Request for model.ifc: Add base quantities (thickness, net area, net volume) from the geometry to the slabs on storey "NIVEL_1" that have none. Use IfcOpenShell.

First a look at what the model holds.

```python
import ifcopenshell
import ifcopenshell.util.element
import ifcopenshell.util.unit

model = ifcopenshell.open("model.ifc")
print(model.schema)
for unit_type in ("LENGTHUNIT", "AREAUNIT", "VOLUMEUNIT"):
    print(unit_type, ifcopenshell.util.unit.calculate_unit_scale(model, unit_type))
storey = next(s for s in model.by_type("IfcBuildingStorey") if s.Name == "NIVEL_1")
slabs = [e for e in ifcopenshell.util.element.get_decomposition(storey) if e.is_a("IfcSlab")]
for e in sorted(slabs, key=lambda e: e.id()):
    print(e.id(), e.is_a(), e.Name, list(ifcopenshell.util.element.get_psets(e, qtos_only=True)), sep=" | ")
```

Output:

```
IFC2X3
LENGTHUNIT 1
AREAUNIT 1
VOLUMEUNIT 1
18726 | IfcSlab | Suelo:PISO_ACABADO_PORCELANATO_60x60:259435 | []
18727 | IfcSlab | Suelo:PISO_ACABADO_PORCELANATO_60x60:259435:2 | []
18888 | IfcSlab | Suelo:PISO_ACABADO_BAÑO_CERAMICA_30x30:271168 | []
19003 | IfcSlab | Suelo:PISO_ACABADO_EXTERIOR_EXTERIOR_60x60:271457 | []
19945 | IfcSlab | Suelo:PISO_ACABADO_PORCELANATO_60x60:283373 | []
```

```python
import ifcopenshell
import ifcopenshell.api.pset
import ifcopenshell.geom
import ifcopenshell.util.element
import ifcopenshell.util.shape
import ifcopenshell.util.unit

model = ifcopenshell.open("model.ifc")
unit_scale = ifcopenshell.util.unit.calculate_unit_scale(model)
area_scale = ifcopenshell.util.unit.calculate_unit_scale(model, "AREAUNIT")
volume_scale = ifcopenshell.util.unit.calculate_unit_scale(model, "VOLUMEUNIT")
settings = ifcopenshell.geom.settings()

storey = next(s for s in model.by_type("IfcBuildingStorey") if s.Name == "NIVEL_1")
slabs = [e for e in ifcopenshell.util.element.get_decomposition(storey) if e.is_a("IfcSlab")]

for e in sorted(slabs, key=lambda e: e.id()):
    if ifcopenshell.util.element.get_psets(e, qtos_only=True, should_inherit=False):
        continue
    # Geometry comes back in metres, in the element's own axes.
    shape = ifcopenshell.geom.create_shape(settings, e)
    values = {
        "Width": ifcopenshell.util.shape.get_z(shape.geometry) / unit_scale,
        "NetArea": ifcopenshell.util.shape.get_footprint_area(shape.geometry) / area_scale,
        "NetVolume": ifcopenshell.util.shape.get_volume(shape.geometry) / volume_scale,
    }
    qto = ifcopenshell.api.pset.add_qto(model, product=e, name="BaseQuantities")
    ifcopenshell.api.pset.edit_qto(model, qto=qto, properties=values)
    print(e.id(), {k: round(v, 3) for k, v in values.items()})

model.write("model_rev.ifc")
```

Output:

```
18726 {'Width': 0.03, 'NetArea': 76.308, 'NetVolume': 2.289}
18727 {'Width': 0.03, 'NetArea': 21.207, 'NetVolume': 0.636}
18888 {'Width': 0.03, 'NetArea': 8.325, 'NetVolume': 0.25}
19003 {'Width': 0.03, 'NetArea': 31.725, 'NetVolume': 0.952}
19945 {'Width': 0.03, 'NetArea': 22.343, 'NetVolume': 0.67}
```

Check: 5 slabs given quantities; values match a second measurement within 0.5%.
